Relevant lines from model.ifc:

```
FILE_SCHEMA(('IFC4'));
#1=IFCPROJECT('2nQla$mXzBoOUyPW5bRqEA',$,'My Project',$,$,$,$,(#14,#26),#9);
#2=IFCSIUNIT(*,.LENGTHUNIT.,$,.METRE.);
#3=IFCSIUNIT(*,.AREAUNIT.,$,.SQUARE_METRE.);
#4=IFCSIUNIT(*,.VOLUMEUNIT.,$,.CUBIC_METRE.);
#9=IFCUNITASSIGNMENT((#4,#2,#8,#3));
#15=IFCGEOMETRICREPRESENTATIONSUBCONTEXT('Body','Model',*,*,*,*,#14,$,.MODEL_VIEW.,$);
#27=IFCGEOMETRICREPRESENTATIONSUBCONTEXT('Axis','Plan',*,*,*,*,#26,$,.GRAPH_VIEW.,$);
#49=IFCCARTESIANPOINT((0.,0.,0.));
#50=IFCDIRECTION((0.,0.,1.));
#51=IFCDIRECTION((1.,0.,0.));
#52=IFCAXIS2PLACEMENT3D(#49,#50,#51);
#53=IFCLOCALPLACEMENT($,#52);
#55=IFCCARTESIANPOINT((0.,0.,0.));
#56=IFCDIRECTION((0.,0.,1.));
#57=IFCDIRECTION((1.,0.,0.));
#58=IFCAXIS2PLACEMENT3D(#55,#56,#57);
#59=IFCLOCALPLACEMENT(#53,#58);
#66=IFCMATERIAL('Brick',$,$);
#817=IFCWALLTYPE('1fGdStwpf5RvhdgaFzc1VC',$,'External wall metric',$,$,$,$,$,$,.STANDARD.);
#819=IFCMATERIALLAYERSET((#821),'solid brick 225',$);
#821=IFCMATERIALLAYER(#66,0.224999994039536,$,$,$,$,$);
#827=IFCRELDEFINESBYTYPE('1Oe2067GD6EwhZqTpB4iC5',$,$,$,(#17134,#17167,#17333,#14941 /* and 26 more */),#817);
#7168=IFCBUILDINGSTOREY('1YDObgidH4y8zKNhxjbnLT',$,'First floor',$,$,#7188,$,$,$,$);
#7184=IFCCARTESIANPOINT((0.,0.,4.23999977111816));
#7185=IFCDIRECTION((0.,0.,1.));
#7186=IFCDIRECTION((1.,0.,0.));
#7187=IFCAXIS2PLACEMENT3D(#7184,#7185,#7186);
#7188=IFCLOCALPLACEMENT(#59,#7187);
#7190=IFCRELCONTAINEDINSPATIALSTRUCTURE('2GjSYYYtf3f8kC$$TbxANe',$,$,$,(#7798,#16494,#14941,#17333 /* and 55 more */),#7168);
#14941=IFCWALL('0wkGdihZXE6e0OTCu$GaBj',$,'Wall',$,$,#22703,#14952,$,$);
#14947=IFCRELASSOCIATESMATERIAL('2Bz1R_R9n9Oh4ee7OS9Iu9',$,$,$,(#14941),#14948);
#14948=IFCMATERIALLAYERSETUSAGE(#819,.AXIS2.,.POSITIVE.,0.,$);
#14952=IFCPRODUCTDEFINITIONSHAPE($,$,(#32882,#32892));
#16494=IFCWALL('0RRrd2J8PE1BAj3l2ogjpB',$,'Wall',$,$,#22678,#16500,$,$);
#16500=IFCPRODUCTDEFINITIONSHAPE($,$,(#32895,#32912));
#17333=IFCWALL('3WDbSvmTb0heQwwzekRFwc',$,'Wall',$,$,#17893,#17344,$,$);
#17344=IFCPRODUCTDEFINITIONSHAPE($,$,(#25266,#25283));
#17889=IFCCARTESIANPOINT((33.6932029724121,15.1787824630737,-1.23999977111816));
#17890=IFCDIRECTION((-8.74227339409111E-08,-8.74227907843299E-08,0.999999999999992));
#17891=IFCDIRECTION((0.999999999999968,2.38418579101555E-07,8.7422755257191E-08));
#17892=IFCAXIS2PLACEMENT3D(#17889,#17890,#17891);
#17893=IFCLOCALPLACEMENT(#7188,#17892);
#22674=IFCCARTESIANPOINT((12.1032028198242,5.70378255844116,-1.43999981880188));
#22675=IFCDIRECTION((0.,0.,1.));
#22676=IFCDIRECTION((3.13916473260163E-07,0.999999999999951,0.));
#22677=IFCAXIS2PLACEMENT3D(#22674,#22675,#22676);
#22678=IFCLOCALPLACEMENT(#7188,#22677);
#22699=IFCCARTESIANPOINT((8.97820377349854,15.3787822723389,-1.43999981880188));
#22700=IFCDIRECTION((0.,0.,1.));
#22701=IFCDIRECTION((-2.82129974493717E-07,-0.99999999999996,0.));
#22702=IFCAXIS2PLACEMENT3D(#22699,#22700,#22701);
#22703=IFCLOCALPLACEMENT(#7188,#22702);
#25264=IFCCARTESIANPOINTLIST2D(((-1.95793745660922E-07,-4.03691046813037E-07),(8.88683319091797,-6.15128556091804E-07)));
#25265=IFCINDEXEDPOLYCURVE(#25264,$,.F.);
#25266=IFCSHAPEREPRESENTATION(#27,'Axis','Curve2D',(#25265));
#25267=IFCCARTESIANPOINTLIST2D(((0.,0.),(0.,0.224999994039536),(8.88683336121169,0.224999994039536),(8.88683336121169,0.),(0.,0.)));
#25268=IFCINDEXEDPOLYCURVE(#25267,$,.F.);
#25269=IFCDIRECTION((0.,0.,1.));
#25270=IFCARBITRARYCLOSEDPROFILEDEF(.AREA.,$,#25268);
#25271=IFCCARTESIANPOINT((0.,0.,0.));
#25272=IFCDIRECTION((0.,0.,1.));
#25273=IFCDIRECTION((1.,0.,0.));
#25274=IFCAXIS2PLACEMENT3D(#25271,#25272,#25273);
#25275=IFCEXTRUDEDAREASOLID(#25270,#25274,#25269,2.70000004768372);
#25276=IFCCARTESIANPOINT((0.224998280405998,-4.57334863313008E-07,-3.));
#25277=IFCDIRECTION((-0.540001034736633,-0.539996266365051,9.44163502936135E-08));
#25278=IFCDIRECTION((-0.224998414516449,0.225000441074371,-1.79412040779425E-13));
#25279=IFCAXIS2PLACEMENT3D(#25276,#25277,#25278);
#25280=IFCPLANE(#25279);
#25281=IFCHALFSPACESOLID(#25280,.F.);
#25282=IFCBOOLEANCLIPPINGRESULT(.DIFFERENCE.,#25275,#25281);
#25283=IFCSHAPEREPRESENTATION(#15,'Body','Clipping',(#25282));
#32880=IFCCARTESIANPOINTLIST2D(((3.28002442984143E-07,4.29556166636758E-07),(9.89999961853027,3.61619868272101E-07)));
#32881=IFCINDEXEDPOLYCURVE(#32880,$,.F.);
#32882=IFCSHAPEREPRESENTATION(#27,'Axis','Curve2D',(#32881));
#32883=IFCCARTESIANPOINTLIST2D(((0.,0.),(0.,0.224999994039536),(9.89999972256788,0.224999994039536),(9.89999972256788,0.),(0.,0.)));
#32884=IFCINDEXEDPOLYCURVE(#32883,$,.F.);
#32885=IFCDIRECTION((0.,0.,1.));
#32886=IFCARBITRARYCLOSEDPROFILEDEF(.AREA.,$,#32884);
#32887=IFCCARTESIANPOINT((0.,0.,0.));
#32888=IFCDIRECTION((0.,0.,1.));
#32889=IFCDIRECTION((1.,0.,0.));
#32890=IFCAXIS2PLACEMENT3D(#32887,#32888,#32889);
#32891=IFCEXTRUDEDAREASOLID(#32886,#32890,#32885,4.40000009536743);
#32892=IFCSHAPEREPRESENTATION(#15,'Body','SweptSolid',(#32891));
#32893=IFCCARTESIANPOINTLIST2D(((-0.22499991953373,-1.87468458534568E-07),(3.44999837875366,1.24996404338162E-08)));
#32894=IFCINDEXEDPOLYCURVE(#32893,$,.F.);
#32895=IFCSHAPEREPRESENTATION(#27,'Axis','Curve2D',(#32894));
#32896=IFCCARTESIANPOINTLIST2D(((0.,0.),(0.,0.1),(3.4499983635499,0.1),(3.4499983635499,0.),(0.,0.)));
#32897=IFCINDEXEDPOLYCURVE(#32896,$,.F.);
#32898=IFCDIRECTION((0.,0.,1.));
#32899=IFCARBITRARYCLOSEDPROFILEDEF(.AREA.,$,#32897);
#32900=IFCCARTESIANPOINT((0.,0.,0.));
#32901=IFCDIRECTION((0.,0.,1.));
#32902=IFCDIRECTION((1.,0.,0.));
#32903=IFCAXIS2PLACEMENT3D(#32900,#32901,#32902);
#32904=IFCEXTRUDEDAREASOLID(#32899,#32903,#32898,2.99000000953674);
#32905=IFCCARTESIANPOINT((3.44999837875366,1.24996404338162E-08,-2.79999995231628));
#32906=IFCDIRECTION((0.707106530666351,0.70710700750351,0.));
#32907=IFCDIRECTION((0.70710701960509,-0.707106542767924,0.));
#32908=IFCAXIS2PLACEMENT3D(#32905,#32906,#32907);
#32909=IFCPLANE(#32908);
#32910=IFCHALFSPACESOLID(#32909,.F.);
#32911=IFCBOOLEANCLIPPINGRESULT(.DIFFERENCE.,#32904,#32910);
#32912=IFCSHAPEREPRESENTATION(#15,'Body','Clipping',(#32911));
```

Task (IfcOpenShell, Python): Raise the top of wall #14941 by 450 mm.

```python
import ifcopenshell
import ifcopenshell.geom
import ifcopenshell.util.representation
import ifcopenshell.util.shape

model = ifcopenshell.open("model.ifc")
settings = ifcopenshell.geom.settings()


def volume(element):
    """Net volume in cubic metres, openings subtracted."""
    shape = ifcopenshell.geom.create_shape(settings, element)
    return ifcopenshell.util.shape.get_volume(shape.geometry)


wall = model.by_guid("0wkGdihZXE6e0OTCu$GaBj")
before = volume(wall)

body = ifcopenshell.util.representation.get_representation(wall, "Model", "Body")
solid = body.Items[0]
old_height = solid.Depth
solid.Depth += 0.45
after = volume(wall)

print(f"height {old_height:g} -> {solid.Depth:g}, volume {before:.3f} -> {after:.3f} m3")

model.write("model-out.ifc")
```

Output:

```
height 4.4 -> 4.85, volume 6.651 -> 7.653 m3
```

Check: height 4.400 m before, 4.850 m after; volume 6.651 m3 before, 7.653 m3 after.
